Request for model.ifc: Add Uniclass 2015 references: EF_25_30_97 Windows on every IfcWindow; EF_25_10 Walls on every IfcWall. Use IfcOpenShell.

First a look at what the model holds.

```python
import ifcopenshell

model = ifcopenshell.open("model.ifc")
print(model.schema)
print("classifications:", [c.Name for c in model.by_type("IfcClassification")])
for ifc_class in ("IfcDoor", "IfcRoof", "IfcStair", "IfcWall", "IfcWindow"):
    print(ifc_class, len(model.by_type(ifc_class)))
```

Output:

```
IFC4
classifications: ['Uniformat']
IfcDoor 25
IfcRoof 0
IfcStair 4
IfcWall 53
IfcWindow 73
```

```python
import ifcopenshell
import ifcopenshell.api.classification

model = ifcopenshell.open("model.ifc")

system = ifcopenshell.api.classification.add_classification(model, classification="Uniclass 2015")

codes = {
    "IfcWindow": ("EF_25_30_97", "Windows"),
    "IfcWall": ("EF_25_10", "Walls"),
}
for ifc_class, (code, name) in codes.items():
    products = model.by_type(ifc_class)
    ifcopenshell.api.classification.add_reference(
        model, products=products, classification=system, identification=code, name=name
    )
    print(code, len(products))

model.write("model_v2.ifc")
```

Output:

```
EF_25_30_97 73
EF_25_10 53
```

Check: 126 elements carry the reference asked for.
